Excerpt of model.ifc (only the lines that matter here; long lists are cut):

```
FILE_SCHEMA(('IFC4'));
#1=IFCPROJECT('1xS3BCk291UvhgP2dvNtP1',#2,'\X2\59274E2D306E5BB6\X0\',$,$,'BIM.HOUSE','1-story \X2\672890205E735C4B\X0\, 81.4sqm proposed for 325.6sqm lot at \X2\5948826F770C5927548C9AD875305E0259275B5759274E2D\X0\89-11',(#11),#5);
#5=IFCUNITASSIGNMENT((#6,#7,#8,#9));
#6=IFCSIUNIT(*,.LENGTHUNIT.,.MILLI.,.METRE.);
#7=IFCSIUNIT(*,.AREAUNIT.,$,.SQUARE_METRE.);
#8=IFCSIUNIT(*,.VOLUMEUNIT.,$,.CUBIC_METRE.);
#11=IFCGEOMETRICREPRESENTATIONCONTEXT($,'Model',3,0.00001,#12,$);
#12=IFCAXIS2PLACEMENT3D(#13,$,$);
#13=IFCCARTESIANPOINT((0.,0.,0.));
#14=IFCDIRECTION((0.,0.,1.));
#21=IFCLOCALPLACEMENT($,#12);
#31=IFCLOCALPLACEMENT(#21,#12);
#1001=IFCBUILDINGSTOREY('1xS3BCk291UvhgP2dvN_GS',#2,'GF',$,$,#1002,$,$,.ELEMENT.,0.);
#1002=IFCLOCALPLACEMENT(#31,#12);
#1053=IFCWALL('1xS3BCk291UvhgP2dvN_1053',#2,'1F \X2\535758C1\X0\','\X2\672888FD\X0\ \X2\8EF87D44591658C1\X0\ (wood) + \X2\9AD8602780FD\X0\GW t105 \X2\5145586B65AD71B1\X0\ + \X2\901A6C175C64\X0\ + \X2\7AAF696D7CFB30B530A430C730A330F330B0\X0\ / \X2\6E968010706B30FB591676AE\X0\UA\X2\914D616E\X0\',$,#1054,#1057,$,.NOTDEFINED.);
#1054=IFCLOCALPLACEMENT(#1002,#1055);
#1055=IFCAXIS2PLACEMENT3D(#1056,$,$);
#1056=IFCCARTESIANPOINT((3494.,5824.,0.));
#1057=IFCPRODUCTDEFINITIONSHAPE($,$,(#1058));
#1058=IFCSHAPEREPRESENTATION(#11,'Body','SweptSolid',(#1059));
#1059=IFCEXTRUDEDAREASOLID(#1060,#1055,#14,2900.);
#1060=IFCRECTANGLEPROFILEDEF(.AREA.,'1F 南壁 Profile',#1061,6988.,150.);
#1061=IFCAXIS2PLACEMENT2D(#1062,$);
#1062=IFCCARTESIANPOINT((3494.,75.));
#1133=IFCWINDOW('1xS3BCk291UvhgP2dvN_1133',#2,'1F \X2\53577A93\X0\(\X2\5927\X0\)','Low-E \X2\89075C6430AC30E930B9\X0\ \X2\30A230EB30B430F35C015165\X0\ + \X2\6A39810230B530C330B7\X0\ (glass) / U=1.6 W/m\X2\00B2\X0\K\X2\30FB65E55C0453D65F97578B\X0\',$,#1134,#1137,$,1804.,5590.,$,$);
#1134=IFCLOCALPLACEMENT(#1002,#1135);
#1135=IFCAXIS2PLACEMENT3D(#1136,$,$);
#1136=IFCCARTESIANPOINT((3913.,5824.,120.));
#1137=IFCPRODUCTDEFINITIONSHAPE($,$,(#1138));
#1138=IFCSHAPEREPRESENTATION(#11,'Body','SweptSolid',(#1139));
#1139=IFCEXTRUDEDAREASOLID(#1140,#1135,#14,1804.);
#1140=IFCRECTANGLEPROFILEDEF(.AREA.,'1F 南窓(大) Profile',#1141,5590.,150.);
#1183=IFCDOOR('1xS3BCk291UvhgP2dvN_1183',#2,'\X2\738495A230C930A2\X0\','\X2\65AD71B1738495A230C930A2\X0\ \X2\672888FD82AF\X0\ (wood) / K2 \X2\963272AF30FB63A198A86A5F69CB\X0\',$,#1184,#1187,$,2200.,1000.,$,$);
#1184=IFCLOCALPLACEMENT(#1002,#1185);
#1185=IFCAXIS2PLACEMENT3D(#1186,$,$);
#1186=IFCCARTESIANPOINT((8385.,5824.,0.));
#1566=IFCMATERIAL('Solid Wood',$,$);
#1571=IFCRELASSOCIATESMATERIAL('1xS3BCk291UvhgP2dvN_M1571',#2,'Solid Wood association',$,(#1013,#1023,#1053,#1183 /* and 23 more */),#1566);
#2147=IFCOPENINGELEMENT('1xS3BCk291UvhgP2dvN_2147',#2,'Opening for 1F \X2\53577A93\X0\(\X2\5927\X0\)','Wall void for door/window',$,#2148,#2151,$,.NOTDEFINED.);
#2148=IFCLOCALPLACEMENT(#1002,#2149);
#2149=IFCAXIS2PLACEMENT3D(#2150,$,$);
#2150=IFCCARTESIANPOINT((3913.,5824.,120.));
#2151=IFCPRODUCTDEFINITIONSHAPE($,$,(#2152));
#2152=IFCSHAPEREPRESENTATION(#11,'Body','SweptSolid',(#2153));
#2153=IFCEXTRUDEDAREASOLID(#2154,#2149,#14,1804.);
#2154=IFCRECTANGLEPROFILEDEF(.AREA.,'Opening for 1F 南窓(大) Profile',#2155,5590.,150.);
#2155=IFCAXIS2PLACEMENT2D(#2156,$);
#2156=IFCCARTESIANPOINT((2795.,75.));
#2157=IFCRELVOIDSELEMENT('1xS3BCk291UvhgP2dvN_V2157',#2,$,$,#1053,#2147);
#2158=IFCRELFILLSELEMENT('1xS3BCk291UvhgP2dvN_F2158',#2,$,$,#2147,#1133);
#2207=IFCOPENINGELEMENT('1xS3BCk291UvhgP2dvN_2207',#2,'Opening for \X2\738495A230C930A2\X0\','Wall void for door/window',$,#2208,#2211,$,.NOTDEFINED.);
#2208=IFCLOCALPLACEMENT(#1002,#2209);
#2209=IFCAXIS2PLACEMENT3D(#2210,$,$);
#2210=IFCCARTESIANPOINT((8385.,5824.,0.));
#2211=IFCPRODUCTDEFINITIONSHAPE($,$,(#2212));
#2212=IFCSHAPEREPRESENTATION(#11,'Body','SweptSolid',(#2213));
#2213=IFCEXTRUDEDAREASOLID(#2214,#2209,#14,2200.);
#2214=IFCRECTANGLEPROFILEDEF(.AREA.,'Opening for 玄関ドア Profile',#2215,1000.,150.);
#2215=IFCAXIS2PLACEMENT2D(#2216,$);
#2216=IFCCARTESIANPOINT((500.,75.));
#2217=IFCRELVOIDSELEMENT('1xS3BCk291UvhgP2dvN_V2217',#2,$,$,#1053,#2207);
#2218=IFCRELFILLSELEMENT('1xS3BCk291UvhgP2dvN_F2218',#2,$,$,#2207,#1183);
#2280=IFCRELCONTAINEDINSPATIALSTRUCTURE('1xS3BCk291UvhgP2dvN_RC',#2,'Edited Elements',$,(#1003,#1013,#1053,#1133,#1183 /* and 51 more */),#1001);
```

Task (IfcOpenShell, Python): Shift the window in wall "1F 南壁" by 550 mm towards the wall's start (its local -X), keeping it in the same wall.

```python
import ifcopenshell
import ifcopenshell.api.geometry
import ifcopenshell.util.placement
import ifcopenshell.util.unit

model = ifcopenshell.open("model.ifc")
unit_scale = ifcopenshell.util.unit.calculate_unit_scale(model)

window = model.by_guid("1xS3BCk291UvhgP2dvN_1133")
opening = window.FillsVoids[0].RelatingOpeningElement
wall = opening.VoidsElements[0].RelatingBuildingElement

wall_matrix = ifcopenshell.util.placement.get_local_placement(wall.ObjectPlacement)
shift = wall_matrix[:3, 0] * -0.55 / unit_scale
before = ifcopenshell.util.placement.get_local_placement(window.ObjectPlacement)[:3, 3].copy()

# The window is not placed relative to its opening, so move both.
for product in (opening, window):
    matrix = ifcopenshell.util.placement.get_local_placement(product.ObjectPlacement)
    matrix[:3, 3] += shift
    ifcopenshell.api.geometry.edit_object_placement(model, product=product, matrix=matrix, is_si=False)

after = ifcopenshell.util.placement.get_local_placement(window.ObjectPlacement)[:3, 3]
print("window moved by", (after - before).round(3) + 0.0)

model.write("model_rev.ifc")
```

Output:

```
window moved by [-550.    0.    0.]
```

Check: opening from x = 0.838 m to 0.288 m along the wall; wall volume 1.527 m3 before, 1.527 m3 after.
